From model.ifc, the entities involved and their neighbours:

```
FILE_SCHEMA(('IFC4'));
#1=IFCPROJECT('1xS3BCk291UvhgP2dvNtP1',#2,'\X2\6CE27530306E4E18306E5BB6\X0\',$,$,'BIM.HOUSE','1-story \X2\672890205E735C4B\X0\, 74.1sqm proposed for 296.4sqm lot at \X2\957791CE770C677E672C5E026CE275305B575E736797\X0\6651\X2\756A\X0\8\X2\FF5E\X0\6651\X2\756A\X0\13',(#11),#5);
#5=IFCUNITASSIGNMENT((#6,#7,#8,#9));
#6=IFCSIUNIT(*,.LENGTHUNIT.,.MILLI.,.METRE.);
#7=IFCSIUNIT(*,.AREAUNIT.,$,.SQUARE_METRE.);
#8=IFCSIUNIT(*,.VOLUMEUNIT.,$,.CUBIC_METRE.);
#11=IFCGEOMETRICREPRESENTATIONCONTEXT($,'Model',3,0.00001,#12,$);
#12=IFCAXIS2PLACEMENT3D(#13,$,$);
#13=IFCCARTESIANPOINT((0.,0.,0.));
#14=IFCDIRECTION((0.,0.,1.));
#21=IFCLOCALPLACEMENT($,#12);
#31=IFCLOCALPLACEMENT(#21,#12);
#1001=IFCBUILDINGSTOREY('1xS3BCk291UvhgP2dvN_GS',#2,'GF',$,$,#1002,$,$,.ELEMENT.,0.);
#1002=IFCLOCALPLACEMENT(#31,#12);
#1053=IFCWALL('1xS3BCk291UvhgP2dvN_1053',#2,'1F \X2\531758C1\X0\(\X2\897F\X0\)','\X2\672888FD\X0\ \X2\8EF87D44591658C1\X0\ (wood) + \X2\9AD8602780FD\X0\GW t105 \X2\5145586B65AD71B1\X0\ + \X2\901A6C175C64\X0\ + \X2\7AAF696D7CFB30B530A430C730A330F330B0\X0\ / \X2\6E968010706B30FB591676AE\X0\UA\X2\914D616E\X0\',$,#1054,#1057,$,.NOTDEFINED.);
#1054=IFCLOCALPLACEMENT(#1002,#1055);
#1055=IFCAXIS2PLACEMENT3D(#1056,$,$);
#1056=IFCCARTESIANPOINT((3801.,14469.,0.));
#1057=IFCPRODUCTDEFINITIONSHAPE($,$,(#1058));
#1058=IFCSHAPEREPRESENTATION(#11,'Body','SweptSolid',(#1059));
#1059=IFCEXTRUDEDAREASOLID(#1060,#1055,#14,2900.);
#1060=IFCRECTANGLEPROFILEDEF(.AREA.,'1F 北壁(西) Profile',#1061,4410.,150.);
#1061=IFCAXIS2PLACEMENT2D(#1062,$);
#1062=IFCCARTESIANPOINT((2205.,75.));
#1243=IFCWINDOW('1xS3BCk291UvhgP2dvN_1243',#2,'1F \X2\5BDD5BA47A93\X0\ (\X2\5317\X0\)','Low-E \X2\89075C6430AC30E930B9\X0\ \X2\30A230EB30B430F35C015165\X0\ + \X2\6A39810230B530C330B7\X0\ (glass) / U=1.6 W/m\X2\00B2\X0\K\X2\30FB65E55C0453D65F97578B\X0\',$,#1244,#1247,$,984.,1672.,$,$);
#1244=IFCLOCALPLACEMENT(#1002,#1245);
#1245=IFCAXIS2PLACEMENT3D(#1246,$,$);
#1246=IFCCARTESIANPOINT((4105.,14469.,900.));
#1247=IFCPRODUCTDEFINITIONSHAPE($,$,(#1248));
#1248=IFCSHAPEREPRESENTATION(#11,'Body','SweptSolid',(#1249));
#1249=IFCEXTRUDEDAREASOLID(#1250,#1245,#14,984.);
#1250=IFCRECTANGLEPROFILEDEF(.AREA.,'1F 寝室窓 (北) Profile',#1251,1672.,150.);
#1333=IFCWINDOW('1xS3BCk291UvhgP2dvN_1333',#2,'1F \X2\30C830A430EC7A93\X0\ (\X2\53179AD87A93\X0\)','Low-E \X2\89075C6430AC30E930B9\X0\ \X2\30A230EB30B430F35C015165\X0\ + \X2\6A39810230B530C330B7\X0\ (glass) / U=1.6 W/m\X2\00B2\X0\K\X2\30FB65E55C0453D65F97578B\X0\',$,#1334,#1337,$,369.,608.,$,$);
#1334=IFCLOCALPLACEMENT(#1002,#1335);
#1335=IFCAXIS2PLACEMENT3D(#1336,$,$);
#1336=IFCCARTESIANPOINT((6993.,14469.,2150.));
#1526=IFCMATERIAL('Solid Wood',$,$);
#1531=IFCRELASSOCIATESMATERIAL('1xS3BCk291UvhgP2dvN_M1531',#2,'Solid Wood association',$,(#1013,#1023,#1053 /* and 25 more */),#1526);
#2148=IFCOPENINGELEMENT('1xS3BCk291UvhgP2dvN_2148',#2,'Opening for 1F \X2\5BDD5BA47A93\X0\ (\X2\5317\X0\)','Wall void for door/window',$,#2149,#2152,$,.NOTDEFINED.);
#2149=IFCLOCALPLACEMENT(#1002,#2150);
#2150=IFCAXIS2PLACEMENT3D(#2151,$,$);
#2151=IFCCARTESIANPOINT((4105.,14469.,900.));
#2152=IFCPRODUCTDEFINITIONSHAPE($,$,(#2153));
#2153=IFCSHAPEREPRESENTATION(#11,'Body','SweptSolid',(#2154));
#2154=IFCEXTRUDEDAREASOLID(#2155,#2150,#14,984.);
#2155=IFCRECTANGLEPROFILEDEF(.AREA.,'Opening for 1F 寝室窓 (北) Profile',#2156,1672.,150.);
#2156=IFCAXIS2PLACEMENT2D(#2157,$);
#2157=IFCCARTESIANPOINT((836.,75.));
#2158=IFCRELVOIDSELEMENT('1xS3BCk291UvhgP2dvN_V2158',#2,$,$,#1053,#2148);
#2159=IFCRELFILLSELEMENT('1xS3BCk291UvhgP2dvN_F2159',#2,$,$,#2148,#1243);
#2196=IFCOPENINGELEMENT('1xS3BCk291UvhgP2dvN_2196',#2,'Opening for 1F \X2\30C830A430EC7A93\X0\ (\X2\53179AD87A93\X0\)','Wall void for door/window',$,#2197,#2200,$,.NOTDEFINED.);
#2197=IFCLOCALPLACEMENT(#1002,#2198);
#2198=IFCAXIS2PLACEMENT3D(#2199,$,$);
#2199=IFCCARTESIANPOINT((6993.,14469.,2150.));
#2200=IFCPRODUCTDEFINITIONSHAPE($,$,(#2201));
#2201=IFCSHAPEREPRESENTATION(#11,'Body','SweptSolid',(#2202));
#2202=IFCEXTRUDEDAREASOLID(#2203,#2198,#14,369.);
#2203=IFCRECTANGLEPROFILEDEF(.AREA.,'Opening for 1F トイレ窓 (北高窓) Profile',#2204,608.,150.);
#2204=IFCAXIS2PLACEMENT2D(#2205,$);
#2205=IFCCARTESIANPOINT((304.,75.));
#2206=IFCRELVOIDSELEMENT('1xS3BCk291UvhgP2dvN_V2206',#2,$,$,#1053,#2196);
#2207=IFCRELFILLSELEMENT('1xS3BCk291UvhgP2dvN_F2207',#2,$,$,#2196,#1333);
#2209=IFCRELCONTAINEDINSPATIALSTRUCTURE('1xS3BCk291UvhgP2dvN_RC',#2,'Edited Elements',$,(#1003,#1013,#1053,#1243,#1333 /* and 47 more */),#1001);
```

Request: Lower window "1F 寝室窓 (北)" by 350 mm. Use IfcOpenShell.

```python
import numpy as np
import ifcopenshell
import ifcopenshell.api.geometry
import ifcopenshell.util.placement
import ifcopenshell.util.unit

model = ifcopenshell.open("model.ifc")
unit_scale = ifcopenshell.util.unit.calculate_unit_scale(model)

window = model.by_guid("1xS3BCk291UvhgP2dvN_1243")
opening = window.FillsVoids[0].RelatingOpeningElement
dz = -350.0

shift = np.array([0.0, 0.0, dz])
# The window is not placed relative to its opening, so move both.
for product in (opening, window):
    matrix = ifcopenshell.util.placement.get_local_placement(product.ObjectPlacement)
    matrix[:3, 3] += shift
    ifcopenshell.api.geometry.edit_object_placement(model, product=product, matrix=matrix, is_si=False)

print(f"moved by {dz * unit_scale:+.3f} m")

model.write("model_rev.ifc")
```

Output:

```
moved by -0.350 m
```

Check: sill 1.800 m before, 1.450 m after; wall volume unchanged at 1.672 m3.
